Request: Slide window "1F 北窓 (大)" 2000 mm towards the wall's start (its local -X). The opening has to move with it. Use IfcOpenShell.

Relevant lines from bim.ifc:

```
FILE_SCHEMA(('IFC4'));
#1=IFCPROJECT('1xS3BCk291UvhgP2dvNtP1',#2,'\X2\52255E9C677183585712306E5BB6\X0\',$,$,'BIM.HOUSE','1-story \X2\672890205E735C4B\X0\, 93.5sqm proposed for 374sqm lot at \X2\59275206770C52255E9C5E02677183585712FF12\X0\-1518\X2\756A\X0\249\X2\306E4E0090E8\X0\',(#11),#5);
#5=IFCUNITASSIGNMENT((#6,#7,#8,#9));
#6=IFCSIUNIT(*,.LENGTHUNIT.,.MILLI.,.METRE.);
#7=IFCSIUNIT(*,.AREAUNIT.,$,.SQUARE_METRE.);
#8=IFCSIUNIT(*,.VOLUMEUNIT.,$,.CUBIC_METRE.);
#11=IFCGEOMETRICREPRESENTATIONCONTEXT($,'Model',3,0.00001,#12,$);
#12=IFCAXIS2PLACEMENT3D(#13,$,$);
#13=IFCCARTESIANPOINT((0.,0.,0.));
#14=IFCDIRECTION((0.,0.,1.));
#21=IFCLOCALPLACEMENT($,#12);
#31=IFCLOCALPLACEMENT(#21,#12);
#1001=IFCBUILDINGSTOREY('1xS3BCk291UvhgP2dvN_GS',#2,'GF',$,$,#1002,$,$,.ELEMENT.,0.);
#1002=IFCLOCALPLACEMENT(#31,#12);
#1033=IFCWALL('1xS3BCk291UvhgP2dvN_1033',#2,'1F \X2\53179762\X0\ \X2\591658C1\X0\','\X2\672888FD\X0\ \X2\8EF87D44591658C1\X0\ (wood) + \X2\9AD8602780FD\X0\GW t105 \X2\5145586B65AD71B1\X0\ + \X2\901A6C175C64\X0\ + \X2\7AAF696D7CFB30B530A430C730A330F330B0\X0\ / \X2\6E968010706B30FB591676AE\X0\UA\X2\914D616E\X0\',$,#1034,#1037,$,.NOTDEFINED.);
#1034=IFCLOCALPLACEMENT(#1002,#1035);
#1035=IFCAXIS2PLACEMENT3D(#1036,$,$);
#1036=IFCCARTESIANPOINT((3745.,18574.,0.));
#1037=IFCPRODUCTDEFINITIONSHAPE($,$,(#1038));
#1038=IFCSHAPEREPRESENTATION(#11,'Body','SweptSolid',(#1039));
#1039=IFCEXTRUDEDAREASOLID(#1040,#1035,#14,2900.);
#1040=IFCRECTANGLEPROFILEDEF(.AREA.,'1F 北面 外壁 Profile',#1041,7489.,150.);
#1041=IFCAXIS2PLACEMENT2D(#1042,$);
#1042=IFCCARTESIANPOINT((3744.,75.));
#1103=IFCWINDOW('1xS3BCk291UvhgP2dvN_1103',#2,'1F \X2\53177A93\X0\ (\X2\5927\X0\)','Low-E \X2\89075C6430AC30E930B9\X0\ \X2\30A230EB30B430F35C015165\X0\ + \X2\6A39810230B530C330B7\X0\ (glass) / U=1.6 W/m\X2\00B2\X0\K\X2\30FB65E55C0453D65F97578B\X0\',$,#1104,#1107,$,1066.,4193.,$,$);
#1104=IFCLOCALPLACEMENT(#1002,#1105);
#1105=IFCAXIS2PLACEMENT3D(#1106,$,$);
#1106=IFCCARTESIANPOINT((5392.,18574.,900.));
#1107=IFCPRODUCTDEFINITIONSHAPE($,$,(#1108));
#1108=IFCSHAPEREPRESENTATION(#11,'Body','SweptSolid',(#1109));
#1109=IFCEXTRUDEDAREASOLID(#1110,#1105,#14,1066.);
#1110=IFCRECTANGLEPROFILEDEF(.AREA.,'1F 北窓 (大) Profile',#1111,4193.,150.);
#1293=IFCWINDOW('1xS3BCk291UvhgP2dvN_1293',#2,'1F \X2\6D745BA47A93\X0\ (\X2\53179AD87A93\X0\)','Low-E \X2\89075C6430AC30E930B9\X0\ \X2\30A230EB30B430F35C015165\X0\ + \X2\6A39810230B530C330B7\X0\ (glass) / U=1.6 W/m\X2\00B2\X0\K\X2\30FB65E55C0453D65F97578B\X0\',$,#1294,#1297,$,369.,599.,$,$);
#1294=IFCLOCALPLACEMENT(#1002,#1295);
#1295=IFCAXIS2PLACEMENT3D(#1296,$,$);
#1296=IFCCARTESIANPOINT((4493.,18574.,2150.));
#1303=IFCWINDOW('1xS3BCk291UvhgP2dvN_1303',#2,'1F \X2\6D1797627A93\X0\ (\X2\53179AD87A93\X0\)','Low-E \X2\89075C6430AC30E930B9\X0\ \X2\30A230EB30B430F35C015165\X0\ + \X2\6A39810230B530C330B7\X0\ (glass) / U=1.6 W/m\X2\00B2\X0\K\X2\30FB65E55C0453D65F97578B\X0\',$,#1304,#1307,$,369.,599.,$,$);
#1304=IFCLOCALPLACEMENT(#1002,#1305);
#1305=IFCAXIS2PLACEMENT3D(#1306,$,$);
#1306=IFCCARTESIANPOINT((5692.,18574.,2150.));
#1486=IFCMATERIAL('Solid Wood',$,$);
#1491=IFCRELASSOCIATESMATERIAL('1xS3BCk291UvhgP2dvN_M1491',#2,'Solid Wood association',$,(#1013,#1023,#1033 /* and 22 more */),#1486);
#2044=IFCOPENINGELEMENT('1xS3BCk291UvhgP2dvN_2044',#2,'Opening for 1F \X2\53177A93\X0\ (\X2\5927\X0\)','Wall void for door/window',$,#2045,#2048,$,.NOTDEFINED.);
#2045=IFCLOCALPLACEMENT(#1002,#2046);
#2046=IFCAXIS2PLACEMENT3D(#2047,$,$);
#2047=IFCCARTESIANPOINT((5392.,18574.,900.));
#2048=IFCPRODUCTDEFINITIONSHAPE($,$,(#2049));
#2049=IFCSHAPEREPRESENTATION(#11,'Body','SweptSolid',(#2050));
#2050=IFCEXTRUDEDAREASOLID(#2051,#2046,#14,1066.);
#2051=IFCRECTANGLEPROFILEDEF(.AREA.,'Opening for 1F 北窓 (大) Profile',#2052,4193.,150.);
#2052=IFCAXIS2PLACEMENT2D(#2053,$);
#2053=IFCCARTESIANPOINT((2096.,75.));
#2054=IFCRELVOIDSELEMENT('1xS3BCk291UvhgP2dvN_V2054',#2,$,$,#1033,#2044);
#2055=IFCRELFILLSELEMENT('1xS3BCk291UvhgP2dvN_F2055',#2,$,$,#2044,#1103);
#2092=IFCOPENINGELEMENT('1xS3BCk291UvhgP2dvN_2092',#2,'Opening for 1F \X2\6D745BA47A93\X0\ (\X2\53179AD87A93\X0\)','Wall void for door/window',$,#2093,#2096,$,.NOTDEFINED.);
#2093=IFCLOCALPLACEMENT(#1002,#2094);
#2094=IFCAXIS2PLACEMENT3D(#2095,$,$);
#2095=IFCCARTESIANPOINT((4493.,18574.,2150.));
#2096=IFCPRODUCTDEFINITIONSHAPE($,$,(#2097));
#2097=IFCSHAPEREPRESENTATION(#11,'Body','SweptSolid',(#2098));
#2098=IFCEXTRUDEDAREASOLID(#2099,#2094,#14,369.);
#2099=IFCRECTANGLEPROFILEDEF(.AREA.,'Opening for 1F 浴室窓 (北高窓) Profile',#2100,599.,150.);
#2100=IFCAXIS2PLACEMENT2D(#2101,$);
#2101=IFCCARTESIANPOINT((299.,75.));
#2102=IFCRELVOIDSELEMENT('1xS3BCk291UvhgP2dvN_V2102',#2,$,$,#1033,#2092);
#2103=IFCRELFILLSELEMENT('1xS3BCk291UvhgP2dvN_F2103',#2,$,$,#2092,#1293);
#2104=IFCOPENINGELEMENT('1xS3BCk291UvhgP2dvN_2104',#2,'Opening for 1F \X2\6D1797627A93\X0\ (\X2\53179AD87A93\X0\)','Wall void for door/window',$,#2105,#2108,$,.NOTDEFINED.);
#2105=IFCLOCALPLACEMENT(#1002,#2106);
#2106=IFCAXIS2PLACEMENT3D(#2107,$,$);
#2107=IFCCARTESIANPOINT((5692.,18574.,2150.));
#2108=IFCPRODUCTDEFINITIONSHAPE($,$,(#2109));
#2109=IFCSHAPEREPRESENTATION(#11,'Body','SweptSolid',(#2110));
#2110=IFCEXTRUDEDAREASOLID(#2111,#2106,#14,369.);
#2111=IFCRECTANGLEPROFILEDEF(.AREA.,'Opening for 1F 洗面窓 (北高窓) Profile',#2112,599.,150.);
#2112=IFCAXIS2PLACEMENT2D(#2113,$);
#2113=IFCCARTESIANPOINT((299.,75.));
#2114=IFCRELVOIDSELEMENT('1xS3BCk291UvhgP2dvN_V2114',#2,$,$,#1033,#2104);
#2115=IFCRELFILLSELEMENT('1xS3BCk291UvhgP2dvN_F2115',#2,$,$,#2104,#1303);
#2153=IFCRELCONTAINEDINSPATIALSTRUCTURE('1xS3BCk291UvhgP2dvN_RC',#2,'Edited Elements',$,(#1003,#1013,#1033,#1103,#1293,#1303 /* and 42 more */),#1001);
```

```python
import ifcopenshell
import ifcopenshell.api.geometry
import ifcopenshell.util.placement

model = ifcopenshell.open("bim.ifc")

window = model.by_guid("1xS3BCk291UvhgP2dvN_1103")
opening = window.FillsVoids[0].RelatingOpeningElement
wall = opening.VoidsElements[0].RelatingBuildingElement

wall_matrix = ifcopenshell.util.placement.get_local_placement(wall.ObjectPlacement)
shift = wall_matrix[:3, 0] * -2000.0
before = ifcopenshell.util.placement.get_local_placement(window.ObjectPlacement)[:3, 3].copy()

# The window is not placed relative to its opening, so move both.
for product in (opening, window):
    matrix = ifcopenshell.util.placement.get_local_placement(product.ObjectPlacement)
    matrix[:3, 3] += shift
    ifcopenshell.api.geometry.edit_object_placement(model, product=product, matrix=matrix, is_si=False)

after = ifcopenshell.util.placement.get_local_placement(window.ObjectPlacement)[:3, 3]
print("window moved by", (after - before).round(3) + 0.0)

model.write("bim_edited.ifc")
```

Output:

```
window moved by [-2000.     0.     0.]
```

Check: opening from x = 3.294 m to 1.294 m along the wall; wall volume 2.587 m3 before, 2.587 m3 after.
